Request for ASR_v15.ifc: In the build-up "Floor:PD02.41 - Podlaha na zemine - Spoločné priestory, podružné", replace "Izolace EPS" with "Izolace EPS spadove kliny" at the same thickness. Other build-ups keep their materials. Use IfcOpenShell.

First a look at what the model holds.

```python
import ifcopenshell
import ifcopenshell.util.element

model = ifcopenshell.open("ASR_v15.ifc")
print(model.schema)
for layer_set in model.by_type("IfcMaterialLayerSet"):
    if layer_set.LayerSetName == "Floor:PD02.41 - Podlaha na zemine - Spoločné priestory, podružné":
        for layer in layer_set.MaterialLayers:
            print(layer.id(), layer.Material and layer.Material.Name, layer.LayerThickness, sep=" | ")
        print(len(ifcopenshell.util.element.get_elements_by_material(model, layer_set)), "elements and types use it")
print(sorted(m.Name for m in model.by_type("IfcMaterial") if m.Name)[:60])
```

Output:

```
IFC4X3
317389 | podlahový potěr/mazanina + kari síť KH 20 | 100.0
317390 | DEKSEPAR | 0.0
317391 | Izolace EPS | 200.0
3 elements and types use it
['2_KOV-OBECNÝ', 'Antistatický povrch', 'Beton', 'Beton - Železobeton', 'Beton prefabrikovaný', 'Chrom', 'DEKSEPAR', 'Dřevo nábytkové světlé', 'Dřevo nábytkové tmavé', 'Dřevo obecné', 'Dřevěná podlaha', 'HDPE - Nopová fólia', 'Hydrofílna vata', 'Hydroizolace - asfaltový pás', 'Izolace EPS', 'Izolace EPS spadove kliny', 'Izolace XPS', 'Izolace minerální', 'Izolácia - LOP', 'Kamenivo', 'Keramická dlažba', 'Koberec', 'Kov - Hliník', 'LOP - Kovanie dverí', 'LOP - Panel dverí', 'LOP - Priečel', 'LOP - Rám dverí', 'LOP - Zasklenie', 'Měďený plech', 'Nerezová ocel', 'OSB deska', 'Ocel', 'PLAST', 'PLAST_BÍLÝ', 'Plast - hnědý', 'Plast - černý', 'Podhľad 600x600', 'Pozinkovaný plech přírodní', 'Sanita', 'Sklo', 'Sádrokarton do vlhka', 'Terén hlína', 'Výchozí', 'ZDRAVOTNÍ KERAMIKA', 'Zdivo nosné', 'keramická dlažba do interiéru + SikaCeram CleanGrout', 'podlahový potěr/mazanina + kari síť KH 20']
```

```python
import ifcopenshell
import ifcopenshell.api.material

model = ifcopenshell.open("ASR_v15.ifc")

layer_set = next(s for s in model.by_type("IfcMaterialLayerSet") if s.LayerSetName == "Floor:PD02.41 - Podlaha na zemine - Spoločné priestory, podružné")
layer = next(l for l in layer_set.MaterialLayers if l.Material and l.Material.Name == "Izolace EPS")
material = next(m for m in model.by_type("IfcMaterial") if m.Name == "Izolace EPS spadove kliny")

# Point this one layer at the other material; renaming the old one would change it everywhere.
ifcopenshell.api.material.edit_layer(model, layer=layer, attributes={"Name": material.Name}, material=material)

print([l.Material.Name if l.Material else None for l in layer_set.MaterialLayers])

model.write("ASR_v15-out.ifc")
```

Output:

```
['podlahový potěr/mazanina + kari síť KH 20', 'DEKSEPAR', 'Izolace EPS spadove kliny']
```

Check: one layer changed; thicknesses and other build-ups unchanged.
